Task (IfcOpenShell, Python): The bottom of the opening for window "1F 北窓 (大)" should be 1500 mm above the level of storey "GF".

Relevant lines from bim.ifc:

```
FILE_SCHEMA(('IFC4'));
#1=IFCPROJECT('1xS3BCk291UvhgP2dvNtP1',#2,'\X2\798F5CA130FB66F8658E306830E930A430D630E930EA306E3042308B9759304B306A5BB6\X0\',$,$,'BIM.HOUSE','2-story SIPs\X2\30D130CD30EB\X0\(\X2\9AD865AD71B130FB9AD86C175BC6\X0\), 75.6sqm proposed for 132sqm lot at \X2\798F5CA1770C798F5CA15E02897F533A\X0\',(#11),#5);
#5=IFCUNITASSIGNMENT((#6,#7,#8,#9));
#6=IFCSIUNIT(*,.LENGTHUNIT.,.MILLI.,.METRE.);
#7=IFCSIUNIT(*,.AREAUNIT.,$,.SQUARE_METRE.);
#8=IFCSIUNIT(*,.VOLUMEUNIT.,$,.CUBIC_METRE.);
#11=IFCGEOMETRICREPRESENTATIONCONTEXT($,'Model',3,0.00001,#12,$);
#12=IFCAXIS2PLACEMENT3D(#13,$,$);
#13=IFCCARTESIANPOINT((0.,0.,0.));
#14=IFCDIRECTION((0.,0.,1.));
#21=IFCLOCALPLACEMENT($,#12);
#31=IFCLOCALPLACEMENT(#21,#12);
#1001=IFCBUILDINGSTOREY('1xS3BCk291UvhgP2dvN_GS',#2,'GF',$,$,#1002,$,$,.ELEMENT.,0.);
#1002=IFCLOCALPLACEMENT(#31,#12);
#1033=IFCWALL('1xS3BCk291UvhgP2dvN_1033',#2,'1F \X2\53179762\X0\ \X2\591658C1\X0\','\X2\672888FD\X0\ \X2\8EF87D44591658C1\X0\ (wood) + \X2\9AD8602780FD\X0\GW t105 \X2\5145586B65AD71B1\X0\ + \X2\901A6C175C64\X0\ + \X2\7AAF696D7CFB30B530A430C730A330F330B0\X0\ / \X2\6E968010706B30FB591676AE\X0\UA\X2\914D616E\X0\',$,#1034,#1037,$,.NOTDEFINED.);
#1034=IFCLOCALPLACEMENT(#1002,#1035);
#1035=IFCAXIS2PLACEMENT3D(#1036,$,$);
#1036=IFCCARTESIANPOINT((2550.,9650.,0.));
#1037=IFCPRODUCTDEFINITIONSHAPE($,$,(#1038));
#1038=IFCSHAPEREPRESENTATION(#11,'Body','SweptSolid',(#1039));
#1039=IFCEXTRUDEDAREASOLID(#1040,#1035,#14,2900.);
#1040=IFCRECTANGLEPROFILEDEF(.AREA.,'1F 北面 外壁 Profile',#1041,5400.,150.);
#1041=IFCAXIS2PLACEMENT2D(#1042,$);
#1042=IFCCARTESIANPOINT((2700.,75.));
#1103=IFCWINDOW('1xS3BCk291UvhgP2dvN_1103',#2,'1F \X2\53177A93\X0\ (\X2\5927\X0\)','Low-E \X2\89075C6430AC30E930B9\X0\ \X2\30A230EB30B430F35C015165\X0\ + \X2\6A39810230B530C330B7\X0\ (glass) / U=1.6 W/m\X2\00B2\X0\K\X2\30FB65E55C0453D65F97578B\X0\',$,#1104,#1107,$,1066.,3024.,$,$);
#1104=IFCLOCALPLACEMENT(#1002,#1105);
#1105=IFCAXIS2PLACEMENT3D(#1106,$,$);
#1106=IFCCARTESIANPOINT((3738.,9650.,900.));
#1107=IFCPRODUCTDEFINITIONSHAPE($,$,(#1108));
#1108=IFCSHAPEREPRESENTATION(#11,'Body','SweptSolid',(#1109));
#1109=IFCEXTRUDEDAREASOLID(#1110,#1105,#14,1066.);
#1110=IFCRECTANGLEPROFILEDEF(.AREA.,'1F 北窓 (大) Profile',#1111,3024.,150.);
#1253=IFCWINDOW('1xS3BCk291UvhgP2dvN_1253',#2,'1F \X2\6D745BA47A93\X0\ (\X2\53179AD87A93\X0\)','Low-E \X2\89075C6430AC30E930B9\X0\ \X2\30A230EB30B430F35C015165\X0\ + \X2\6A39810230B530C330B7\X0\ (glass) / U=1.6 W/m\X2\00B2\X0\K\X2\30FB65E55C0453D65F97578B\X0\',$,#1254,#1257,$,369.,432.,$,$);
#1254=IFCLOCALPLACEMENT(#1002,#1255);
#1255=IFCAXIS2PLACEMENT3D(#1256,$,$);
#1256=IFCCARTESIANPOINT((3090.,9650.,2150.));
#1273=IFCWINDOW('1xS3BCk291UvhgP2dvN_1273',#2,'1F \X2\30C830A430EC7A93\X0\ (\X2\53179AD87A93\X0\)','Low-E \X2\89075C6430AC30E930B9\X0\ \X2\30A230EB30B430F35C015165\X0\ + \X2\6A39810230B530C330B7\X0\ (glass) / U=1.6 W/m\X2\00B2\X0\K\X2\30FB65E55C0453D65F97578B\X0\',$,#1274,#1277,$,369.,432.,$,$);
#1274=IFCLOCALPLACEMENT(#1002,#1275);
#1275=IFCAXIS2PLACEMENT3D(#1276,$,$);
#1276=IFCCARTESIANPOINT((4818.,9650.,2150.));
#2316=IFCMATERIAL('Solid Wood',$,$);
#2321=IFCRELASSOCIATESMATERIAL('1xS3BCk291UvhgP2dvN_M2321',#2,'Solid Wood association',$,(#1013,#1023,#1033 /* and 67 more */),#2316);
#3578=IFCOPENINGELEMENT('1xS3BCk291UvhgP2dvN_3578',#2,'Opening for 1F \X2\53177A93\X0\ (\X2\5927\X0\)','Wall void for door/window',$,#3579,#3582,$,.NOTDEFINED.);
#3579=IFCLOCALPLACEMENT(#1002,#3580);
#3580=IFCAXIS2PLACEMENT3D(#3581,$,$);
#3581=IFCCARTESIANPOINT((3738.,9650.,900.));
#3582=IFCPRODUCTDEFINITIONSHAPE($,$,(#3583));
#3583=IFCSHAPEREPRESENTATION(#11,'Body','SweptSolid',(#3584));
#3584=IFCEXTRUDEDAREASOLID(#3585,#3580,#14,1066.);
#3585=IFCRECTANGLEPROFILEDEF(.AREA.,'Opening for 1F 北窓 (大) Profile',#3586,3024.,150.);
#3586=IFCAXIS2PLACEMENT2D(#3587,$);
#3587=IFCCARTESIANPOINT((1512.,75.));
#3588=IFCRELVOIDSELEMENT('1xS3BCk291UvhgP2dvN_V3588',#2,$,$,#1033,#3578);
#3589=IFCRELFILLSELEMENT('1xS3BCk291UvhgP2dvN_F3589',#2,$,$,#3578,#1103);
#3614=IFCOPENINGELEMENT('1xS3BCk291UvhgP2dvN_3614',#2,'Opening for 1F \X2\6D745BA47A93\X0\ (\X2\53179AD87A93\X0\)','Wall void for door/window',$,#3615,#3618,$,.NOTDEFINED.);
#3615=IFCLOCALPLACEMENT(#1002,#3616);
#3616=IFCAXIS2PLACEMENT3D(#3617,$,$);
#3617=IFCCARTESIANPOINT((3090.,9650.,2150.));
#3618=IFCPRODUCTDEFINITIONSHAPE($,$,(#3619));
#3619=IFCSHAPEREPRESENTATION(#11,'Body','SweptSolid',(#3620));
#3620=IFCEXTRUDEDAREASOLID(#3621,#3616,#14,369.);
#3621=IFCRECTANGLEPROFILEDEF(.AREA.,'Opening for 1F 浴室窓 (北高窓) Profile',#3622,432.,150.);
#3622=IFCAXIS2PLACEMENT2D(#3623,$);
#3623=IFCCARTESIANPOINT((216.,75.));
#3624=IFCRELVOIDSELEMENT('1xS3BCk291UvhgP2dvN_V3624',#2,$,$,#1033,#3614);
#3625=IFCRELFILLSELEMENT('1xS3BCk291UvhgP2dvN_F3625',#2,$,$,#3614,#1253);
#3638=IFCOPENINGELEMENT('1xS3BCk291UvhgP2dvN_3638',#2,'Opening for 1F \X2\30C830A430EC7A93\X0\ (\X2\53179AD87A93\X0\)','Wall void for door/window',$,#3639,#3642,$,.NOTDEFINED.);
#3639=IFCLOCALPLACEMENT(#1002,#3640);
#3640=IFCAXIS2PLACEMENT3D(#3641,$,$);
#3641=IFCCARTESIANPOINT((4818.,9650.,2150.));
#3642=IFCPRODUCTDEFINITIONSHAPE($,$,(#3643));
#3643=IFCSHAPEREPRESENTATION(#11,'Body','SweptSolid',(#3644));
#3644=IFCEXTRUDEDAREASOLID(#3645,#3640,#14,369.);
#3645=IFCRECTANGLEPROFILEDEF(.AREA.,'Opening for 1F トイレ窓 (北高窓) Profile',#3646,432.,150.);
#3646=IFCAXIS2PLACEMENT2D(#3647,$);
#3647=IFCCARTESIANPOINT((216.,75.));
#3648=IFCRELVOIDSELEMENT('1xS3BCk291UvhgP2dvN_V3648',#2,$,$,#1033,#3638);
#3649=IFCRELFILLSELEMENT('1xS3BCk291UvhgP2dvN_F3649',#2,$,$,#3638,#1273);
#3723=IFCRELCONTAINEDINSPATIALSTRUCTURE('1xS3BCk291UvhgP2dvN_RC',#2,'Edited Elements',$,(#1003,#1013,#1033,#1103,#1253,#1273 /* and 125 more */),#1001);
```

```python
import numpy as np
import ifcopenshell
import ifcopenshell.api.geometry
import ifcopenshell.geom
import ifcopenshell.util.element
import ifcopenshell.util.placement
import ifcopenshell.util.shape
import ifcopenshell.util.unit

model = ifcopenshell.open("bim.ifc")
unit_scale = ifcopenshell.util.unit.calculate_unit_scale(model)

window = model.by_id(1103)
opening = window.FillsVoids[0].RelatingOpeningElement
storey = ifcopenshell.util.element.get_container(window, ifc_class="IfcBuildingStorey")
level = ifcopenshell.util.placement.get_local_placement(storey.ObjectPlacement)[2, 3]

# The opening's origin need not be at the sill, so measure its lowest point.
shape = ifcopenshell.geom.create_shape(ifcopenshell.geom.settings(), opening)
bottom = ifcopenshell.util.shape.get_shape_bottom_elevation(shape, shape.geometry) / unit_scale
dz = level + 1.5 / unit_scale - bottom

shift = np.array([0.0, 0.0, dz])
# The window is not placed relative to its opening, so move both.
for product in (opening, window):
    matrix = ifcopenshell.util.placement.get_local_placement(product.ObjectPlacement)
    matrix[:3, 3] += shift
    ifcopenshell.api.geometry.edit_object_placement(model, product=product, matrix=matrix, is_si=False)

print(f"moved by {dz * unit_scale:+.3f} m")

model.write("bim_edited.ifc")
```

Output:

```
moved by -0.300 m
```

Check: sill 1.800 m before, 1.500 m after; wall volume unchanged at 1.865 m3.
